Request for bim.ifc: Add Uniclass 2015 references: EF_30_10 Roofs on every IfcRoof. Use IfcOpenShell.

First a look at what the model holds.

```python
import ifcopenshell

model = ifcopenshell.open("bim.ifc")
print(model.schema)
print("classifications:", [c.Name for c in model.by_type("IfcClassification")])
for ifc_class in ("IfcDoor", "IfcRoof", "IfcStair", "IfcWall", "IfcWindow"):
    print(ifc_class, len(model.by_type(ifc_class)))
```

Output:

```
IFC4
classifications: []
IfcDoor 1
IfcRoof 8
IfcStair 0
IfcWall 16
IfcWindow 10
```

```python
import ifcopenshell
import ifcopenshell.api.classification

model = ifcopenshell.open("bim.ifc")

system = ifcopenshell.api.classification.add_classification(model, classification="Uniclass 2015")

codes = {
    "IfcRoof": ("EF_30_10", "Roofs"),
}
for ifc_class, (code, name) in codes.items():
    products = model.by_type(ifc_class)
    ifcopenshell.api.classification.add_reference(
        model, products=products, classification=system, identification=code, name=name
    )
    print(code, len(products))

model.write("bim-out.ifc")
```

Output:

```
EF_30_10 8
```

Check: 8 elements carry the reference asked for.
